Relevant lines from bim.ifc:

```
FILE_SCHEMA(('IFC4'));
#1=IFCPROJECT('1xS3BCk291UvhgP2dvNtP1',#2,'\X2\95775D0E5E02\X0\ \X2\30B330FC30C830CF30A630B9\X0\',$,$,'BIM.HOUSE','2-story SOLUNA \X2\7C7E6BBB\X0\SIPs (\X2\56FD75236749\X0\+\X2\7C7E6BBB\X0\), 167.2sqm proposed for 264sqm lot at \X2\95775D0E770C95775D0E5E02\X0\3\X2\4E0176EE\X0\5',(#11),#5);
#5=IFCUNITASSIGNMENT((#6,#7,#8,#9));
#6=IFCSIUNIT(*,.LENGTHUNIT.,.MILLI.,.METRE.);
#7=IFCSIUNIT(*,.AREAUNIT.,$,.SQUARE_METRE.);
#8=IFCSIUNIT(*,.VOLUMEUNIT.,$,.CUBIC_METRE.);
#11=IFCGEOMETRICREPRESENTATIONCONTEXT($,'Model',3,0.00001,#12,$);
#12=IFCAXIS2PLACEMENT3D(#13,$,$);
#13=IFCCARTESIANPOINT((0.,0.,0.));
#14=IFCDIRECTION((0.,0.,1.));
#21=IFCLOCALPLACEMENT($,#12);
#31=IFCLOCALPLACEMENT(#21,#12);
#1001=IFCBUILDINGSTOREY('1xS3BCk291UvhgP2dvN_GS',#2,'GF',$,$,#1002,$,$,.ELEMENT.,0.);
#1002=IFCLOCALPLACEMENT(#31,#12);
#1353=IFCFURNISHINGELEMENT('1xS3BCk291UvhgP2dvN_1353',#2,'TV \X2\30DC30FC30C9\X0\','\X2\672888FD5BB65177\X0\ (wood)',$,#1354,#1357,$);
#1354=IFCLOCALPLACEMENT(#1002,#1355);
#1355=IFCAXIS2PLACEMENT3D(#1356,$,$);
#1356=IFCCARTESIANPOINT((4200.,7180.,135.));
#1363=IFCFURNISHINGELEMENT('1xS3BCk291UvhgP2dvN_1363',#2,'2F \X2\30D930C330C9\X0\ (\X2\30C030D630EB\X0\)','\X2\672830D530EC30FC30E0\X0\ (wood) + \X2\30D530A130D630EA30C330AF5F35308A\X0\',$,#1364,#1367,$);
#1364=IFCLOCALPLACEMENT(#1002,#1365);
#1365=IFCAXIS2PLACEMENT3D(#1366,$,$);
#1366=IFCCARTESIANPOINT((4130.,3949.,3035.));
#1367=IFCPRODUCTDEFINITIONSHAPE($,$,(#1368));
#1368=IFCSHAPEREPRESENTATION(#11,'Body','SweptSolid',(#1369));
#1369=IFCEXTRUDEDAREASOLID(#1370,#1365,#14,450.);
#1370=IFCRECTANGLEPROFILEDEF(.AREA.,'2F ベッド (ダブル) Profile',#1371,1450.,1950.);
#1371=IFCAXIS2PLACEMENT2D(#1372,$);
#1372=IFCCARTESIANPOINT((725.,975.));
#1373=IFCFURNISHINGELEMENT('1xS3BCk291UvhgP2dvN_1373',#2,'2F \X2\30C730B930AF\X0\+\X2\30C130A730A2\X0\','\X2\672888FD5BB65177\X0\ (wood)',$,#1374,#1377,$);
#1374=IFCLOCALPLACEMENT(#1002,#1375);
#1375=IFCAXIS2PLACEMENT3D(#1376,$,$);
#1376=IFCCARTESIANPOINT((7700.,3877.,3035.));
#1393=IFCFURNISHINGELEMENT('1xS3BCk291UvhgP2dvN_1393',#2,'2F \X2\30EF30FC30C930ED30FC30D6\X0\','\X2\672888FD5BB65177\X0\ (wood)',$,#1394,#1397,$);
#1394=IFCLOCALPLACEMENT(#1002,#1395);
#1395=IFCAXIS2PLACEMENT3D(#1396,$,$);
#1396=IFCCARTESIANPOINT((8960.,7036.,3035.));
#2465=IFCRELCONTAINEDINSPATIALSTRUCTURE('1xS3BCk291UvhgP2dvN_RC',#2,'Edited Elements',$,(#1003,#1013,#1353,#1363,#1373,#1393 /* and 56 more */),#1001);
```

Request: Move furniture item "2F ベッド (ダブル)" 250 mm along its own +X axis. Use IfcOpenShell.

```python
import ifcopenshell
import ifcopenshell.api.geometry
import ifcopenshell.util.placement
import ifcopenshell.util.unit

model = ifcopenshell.open("bim.ifc")
unit_scale = ifcopenshell.util.unit.calculate_unit_scale(model)

item = model.by_guid("1xS3BCk291UvhgP2dvN_1363")
matrix = ifcopenshell.util.placement.get_local_placement(item.ObjectPlacement)
matrix[:3, 3] += matrix[:3, 0] * 0.25 / unit_scale
ifcopenshell.api.geometry.edit_object_placement(model, product=item, matrix=matrix, is_si=False)

print(ifcopenshell.util.placement.get_local_placement(item.ObjectPlacement).round(3) + 0.0)

model.write("bim_updated.ifc")
```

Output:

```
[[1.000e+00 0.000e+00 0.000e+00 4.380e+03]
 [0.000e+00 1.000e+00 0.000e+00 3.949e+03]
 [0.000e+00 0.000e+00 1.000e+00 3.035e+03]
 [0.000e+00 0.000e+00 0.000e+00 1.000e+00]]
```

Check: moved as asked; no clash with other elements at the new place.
